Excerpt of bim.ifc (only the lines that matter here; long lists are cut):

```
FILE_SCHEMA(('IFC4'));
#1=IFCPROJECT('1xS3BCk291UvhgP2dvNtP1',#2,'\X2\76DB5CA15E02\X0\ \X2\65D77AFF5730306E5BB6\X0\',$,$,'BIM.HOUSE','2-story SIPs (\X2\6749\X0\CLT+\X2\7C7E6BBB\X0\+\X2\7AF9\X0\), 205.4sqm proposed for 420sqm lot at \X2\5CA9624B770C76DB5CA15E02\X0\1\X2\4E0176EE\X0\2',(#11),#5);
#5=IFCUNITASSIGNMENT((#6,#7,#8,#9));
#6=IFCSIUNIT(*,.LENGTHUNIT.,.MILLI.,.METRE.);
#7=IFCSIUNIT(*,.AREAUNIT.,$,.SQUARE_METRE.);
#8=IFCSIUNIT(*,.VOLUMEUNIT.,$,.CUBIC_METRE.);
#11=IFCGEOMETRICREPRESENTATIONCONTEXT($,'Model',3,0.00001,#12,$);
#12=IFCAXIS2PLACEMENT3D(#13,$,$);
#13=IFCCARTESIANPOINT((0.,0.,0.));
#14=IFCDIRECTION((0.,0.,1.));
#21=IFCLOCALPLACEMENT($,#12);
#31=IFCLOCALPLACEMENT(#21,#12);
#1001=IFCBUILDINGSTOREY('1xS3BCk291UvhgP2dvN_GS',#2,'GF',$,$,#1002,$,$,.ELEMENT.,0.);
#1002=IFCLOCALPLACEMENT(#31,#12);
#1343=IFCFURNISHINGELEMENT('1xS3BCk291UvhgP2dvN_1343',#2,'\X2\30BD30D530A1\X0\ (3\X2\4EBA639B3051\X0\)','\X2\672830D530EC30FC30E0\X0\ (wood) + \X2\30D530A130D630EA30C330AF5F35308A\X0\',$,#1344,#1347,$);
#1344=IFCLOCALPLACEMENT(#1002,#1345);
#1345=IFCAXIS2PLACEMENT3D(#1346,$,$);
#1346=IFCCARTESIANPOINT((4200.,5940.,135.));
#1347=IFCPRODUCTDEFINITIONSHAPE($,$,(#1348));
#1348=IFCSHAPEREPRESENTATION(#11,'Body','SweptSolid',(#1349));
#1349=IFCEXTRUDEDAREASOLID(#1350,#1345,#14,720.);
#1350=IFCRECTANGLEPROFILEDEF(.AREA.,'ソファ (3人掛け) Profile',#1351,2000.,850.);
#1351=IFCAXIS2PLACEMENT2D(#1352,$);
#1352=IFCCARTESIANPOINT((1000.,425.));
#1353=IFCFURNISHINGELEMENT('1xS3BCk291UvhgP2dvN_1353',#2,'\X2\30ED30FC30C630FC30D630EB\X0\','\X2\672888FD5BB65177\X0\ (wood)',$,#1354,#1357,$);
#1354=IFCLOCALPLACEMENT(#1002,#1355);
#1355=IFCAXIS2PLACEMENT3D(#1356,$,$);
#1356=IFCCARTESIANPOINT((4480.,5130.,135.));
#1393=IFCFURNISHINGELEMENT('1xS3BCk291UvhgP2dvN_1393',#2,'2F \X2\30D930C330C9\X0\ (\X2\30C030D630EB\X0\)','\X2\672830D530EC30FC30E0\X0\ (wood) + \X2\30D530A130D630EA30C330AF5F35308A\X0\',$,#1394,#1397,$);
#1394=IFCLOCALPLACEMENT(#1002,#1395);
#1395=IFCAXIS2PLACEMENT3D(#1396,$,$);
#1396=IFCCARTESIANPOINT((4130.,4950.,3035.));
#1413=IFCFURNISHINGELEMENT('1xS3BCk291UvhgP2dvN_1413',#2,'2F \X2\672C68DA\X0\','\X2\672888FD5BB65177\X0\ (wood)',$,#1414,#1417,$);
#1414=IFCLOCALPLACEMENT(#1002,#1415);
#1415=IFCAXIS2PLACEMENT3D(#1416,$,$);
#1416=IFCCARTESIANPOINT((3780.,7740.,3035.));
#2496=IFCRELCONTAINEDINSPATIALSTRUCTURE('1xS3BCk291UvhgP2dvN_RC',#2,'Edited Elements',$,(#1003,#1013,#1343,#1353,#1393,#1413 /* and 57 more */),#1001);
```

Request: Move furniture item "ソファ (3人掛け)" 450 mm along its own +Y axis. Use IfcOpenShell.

```python
import ifcopenshell
import ifcopenshell.api.geometry
import ifcopenshell.util.placement
import ifcopenshell.util.unit

model = ifcopenshell.open("bim.ifc")
unit_scale = ifcopenshell.util.unit.calculate_unit_scale(model)

item = model.by_id(1343)
matrix = ifcopenshell.util.placement.get_local_placement(item.ObjectPlacement)
matrix[:3, 3] += matrix[:3, 1] * 0.45 / unit_scale
ifcopenshell.api.geometry.edit_object_placement(model, product=item, matrix=matrix, is_si=False)

print(ifcopenshell.util.placement.get_local_placement(item.ObjectPlacement).round(3) + 0.0)

model.write("bim_v2.ifc")
```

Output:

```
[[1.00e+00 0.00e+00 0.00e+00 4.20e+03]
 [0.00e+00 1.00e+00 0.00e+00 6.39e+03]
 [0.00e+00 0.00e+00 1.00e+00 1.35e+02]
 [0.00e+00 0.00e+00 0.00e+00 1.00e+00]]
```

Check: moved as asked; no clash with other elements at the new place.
